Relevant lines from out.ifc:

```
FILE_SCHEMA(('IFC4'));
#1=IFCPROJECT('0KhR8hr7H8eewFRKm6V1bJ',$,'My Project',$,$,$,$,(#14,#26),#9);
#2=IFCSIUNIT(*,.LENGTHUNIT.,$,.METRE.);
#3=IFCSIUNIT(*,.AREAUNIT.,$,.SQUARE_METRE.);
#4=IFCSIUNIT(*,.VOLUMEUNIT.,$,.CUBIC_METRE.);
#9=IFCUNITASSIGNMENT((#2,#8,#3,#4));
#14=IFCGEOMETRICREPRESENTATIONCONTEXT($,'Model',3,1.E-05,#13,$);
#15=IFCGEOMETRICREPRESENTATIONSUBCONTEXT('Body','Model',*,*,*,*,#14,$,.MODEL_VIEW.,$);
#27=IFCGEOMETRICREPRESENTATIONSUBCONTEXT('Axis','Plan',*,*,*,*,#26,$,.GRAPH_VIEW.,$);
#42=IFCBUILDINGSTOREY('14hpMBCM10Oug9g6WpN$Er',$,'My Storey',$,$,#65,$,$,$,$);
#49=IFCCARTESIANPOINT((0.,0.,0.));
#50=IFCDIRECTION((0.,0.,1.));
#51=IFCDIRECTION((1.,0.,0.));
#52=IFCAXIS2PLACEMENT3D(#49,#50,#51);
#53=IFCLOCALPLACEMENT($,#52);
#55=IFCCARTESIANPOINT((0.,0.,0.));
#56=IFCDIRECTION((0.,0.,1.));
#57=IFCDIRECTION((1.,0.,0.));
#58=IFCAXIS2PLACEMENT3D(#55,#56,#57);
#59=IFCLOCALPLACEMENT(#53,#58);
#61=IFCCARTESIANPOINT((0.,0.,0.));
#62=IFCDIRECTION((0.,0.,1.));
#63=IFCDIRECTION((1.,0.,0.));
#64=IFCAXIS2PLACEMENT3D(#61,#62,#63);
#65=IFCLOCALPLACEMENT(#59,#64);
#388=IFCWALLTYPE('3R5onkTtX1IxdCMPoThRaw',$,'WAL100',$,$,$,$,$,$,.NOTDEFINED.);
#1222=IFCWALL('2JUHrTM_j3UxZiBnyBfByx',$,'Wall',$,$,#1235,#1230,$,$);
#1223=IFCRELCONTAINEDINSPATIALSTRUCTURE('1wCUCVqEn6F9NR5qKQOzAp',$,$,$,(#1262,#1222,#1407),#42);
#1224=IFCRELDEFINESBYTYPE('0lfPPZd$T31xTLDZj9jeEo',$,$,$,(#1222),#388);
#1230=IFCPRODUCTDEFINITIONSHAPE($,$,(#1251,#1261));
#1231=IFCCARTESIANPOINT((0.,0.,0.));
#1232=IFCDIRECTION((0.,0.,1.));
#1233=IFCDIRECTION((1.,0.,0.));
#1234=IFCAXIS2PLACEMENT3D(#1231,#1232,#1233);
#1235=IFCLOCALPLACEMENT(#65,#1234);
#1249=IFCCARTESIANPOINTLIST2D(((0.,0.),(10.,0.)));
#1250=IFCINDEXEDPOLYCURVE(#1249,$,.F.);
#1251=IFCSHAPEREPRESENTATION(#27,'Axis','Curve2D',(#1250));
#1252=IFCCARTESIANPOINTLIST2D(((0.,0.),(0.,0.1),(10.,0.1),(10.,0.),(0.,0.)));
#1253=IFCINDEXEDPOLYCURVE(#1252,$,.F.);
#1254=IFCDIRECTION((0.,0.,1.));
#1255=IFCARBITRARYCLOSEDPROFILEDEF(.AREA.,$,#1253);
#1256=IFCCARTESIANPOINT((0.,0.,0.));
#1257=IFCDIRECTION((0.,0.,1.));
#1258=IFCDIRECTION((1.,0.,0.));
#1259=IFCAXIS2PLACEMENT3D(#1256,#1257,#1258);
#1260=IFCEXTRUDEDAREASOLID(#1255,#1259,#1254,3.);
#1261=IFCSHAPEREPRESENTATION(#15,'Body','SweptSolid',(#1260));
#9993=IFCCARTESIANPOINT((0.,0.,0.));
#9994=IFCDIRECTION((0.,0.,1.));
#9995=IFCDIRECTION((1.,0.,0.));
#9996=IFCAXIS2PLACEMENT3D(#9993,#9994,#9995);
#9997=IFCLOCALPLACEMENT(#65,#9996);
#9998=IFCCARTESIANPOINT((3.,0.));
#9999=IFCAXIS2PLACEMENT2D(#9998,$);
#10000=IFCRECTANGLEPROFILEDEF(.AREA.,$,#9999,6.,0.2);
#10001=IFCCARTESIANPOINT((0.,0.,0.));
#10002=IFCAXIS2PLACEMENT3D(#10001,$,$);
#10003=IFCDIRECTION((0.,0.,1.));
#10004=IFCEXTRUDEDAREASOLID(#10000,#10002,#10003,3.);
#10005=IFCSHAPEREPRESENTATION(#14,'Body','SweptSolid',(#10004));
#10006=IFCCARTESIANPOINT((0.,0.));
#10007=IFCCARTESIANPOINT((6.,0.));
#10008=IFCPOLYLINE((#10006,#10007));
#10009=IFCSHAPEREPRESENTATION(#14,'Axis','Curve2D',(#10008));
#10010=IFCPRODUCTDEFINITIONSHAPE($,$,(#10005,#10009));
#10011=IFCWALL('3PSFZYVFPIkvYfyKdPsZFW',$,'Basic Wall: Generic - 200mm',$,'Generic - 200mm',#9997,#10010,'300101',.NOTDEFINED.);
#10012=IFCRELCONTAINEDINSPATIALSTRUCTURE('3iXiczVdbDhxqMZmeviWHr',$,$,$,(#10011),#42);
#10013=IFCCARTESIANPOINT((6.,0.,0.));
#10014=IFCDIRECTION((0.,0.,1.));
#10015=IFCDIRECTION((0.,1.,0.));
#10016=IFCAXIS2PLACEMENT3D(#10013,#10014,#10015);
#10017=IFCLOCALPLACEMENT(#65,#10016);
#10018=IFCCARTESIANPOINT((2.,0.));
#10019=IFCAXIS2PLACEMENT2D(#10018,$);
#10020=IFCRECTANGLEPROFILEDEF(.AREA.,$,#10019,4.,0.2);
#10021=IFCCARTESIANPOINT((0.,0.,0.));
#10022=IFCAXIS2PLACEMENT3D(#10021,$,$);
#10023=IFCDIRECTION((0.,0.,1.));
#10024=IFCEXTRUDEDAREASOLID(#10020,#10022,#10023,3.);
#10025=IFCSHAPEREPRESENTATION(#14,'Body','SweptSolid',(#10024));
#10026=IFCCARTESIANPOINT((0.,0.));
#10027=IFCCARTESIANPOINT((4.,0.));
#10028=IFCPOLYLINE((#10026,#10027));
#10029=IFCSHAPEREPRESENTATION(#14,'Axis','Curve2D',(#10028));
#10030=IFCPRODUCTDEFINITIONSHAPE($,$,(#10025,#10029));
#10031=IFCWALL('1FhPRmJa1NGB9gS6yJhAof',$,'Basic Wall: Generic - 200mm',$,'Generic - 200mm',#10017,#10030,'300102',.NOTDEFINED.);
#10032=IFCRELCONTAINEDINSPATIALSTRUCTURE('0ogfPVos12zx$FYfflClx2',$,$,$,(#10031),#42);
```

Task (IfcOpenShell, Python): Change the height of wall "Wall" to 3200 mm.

```python
import ifcopenshell
import ifcopenshell.geom
import ifcopenshell.util.representation
import ifcopenshell.util.shape
import ifcopenshell.util.unit

model = ifcopenshell.open("out.ifc")
unit_scale = ifcopenshell.util.unit.calculate_unit_scale(model)
settings = ifcopenshell.geom.settings()


def volume(element):
    """Net volume in cubic metres, openings subtracted."""
    shape = ifcopenshell.geom.create_shape(settings, element)
    return ifcopenshell.util.shape.get_volume(shape.geometry)


wall = model.by_guid("2JUHrTM_j3UxZiBnyBfByx")
before = volume(wall)

body = ifcopenshell.util.representation.get_representation(wall, "Model", "Body")
solid = body.Items[0]
old_height = solid.Depth
solid.Depth = 3.2 / unit_scale
after = volume(wall)

print(f"height {old_height:g} -> {solid.Depth:g}, volume {before:.3f} -> {after:.3f} m3")

model.write("out_v2.ifc")
```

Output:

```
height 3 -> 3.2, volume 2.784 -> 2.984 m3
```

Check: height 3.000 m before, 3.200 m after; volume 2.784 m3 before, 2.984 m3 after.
